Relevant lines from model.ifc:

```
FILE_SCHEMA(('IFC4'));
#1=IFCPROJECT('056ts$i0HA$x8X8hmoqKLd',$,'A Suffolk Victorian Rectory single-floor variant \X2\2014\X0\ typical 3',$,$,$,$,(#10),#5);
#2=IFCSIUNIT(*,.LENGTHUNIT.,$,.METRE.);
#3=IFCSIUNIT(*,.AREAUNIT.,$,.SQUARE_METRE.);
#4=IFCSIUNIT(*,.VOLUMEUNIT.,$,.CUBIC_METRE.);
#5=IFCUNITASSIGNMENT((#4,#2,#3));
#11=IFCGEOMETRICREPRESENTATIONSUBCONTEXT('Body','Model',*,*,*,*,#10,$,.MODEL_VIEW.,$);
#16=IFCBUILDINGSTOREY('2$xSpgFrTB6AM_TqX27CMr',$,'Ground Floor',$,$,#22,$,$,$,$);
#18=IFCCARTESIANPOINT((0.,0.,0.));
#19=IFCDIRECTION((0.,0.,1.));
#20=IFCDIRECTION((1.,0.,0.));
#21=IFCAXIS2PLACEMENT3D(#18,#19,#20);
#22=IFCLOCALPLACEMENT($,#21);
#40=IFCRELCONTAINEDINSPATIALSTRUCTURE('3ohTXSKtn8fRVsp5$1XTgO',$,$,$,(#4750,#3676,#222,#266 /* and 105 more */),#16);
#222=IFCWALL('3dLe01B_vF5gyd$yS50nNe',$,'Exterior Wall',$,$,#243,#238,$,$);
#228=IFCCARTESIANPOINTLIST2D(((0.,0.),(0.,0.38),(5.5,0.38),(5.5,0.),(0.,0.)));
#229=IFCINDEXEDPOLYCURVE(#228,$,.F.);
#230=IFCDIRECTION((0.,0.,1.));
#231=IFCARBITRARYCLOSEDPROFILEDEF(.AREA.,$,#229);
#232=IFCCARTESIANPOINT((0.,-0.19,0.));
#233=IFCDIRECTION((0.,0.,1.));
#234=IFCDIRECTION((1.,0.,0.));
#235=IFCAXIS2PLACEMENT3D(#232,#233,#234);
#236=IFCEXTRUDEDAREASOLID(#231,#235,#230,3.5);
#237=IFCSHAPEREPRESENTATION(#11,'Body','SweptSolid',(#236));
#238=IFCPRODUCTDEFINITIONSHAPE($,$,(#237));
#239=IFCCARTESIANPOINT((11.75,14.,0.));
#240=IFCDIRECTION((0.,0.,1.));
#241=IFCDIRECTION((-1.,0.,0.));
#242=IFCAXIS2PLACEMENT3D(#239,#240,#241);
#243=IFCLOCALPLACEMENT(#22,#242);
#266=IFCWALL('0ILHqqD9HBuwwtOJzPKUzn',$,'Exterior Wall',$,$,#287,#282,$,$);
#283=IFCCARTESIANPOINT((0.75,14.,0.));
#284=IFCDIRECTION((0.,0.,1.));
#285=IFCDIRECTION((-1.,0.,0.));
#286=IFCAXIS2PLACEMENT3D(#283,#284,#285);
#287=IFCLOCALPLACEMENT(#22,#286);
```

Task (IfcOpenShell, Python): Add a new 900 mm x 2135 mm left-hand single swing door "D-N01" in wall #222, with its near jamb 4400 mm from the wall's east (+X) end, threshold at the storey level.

```python
import numpy as np
import ifcopenshell
import ifcopenshell.api.feature
import ifcopenshell.api.geometry
import ifcopenshell.api.root
import ifcopenshell.api.spatial
import ifcopenshell.geom
import ifcopenshell.util.element
import ifcopenshell.util.placement
import ifcopenshell.util.representation
import ifcopenshell.util.shape
import ifcopenshell.util.unit

model = ifcopenshell.open("model.ifc")
unit_scale = ifcopenshell.util.unit.calculate_unit_scale(model)
settings = ifcopenshell.geom.settings()


def volume(element):
    """Net volume in cubic metres, openings subtracted."""
    shape = ifcopenshell.geom.create_shape(settings, element)
    return ifcopenshell.util.shape.get_volume(shape.geometry)


wall = model.by_id(222)
storey = ifcopenshell.util.element.get_container(wall, ifc_class="IfcBuildingStorey")
context = ifcopenshell.util.representation.get_context(model, "Model", "Body", "MODEL_VIEW")
before = volume(wall)

width, height, from_end, sill = 0.9, 2.135, 4.4, 0.0  # metres

# The wall runs along its own X axis, and the end named is its -X end.
wall_shape = ifcopenshell.geom.create_shape(settings, wall)
x, y, z = ifcopenshell.util.shape.get_vertices(wall_shape.geometry).T
start = x.min() + from_end
face, thickness = float(y.min()), float(y.max() - y.min())
wall_matrix = ifcopenshell.util.placement.get_local_placement(wall.ObjectPlacement)
level = ifcopenshell.util.placement.get_local_placement(storey.ObjectPlacement)[2, 3]


def in_wall(x, y):
    """Placement at x, y metres in the wall's axes, at sill height."""
    matrix = wall_matrix.copy()
    matrix[:, 3] = wall_matrix @ np.array([x / unit_scale, y / unit_scale, 0.0, 1.0])
    matrix[2, 3] = level + sill / unit_scale
    return matrix


# Opening: a box that overshoots both wall faces by 50 mm.
opening = ifcopenshell.api.root.create_entity(model, ifc_class="IfcOpeningElement", predefined_type="OPENING")
box = ifcopenshell.api.geometry.add_wall_representation(
    model, context=context, length=width, height=height, thickness=thickness + 0.1
)
ifcopenshell.api.geometry.assign_representation(model, product=opening, representation=box)
ifcopenshell.api.geometry.edit_object_placement(model, product=opening, matrix=in_wall(start, face - 0.05), is_si=False)
ifcopenshell.api.feature.add_feature(model, feature=opening, element=wall)

door = ifcopenshell.api.root.create_entity(model, ifc_class="IfcDoor", name="D-N01", predefined_type="DOOR")
door.OverallWidth, door.OverallHeight = width / unit_scale, height / unit_scale
door.OperationType = "SINGLE_SWING_LEFT"
body = ifcopenshell.api.geometry.add_door_representation(
    model,
    context=context,
    overall_width=door.OverallWidth,
    overall_height=door.OverallHeight,
    operation_type="SINGLE_SWING_LEFT",
    lining_properties={"LiningDepth": thickness / unit_scale, "ThresholdDepth": thickness / unit_scale},
)
ifcopenshell.api.geometry.assign_representation(model, product=door, representation=body)
ifcopenshell.api.spatial.assign_container(model, products=[door], relating_structure=storey)
ifcopenshell.api.feature.add_filling(model, opening=opening, element=door)

# The lining spans the wall, so the door starts at the wall face.
ifcopenshell.api.geometry.edit_object_placement(model, product=door, matrix=in_wall(start, face), is_si=False)

after = volume(wall)

print(f"wall volume {before:.3f} -> {after:.3f} m3")

model.write("model_edited.ifc")
```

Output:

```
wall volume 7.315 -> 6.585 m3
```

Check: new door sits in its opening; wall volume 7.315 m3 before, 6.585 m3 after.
